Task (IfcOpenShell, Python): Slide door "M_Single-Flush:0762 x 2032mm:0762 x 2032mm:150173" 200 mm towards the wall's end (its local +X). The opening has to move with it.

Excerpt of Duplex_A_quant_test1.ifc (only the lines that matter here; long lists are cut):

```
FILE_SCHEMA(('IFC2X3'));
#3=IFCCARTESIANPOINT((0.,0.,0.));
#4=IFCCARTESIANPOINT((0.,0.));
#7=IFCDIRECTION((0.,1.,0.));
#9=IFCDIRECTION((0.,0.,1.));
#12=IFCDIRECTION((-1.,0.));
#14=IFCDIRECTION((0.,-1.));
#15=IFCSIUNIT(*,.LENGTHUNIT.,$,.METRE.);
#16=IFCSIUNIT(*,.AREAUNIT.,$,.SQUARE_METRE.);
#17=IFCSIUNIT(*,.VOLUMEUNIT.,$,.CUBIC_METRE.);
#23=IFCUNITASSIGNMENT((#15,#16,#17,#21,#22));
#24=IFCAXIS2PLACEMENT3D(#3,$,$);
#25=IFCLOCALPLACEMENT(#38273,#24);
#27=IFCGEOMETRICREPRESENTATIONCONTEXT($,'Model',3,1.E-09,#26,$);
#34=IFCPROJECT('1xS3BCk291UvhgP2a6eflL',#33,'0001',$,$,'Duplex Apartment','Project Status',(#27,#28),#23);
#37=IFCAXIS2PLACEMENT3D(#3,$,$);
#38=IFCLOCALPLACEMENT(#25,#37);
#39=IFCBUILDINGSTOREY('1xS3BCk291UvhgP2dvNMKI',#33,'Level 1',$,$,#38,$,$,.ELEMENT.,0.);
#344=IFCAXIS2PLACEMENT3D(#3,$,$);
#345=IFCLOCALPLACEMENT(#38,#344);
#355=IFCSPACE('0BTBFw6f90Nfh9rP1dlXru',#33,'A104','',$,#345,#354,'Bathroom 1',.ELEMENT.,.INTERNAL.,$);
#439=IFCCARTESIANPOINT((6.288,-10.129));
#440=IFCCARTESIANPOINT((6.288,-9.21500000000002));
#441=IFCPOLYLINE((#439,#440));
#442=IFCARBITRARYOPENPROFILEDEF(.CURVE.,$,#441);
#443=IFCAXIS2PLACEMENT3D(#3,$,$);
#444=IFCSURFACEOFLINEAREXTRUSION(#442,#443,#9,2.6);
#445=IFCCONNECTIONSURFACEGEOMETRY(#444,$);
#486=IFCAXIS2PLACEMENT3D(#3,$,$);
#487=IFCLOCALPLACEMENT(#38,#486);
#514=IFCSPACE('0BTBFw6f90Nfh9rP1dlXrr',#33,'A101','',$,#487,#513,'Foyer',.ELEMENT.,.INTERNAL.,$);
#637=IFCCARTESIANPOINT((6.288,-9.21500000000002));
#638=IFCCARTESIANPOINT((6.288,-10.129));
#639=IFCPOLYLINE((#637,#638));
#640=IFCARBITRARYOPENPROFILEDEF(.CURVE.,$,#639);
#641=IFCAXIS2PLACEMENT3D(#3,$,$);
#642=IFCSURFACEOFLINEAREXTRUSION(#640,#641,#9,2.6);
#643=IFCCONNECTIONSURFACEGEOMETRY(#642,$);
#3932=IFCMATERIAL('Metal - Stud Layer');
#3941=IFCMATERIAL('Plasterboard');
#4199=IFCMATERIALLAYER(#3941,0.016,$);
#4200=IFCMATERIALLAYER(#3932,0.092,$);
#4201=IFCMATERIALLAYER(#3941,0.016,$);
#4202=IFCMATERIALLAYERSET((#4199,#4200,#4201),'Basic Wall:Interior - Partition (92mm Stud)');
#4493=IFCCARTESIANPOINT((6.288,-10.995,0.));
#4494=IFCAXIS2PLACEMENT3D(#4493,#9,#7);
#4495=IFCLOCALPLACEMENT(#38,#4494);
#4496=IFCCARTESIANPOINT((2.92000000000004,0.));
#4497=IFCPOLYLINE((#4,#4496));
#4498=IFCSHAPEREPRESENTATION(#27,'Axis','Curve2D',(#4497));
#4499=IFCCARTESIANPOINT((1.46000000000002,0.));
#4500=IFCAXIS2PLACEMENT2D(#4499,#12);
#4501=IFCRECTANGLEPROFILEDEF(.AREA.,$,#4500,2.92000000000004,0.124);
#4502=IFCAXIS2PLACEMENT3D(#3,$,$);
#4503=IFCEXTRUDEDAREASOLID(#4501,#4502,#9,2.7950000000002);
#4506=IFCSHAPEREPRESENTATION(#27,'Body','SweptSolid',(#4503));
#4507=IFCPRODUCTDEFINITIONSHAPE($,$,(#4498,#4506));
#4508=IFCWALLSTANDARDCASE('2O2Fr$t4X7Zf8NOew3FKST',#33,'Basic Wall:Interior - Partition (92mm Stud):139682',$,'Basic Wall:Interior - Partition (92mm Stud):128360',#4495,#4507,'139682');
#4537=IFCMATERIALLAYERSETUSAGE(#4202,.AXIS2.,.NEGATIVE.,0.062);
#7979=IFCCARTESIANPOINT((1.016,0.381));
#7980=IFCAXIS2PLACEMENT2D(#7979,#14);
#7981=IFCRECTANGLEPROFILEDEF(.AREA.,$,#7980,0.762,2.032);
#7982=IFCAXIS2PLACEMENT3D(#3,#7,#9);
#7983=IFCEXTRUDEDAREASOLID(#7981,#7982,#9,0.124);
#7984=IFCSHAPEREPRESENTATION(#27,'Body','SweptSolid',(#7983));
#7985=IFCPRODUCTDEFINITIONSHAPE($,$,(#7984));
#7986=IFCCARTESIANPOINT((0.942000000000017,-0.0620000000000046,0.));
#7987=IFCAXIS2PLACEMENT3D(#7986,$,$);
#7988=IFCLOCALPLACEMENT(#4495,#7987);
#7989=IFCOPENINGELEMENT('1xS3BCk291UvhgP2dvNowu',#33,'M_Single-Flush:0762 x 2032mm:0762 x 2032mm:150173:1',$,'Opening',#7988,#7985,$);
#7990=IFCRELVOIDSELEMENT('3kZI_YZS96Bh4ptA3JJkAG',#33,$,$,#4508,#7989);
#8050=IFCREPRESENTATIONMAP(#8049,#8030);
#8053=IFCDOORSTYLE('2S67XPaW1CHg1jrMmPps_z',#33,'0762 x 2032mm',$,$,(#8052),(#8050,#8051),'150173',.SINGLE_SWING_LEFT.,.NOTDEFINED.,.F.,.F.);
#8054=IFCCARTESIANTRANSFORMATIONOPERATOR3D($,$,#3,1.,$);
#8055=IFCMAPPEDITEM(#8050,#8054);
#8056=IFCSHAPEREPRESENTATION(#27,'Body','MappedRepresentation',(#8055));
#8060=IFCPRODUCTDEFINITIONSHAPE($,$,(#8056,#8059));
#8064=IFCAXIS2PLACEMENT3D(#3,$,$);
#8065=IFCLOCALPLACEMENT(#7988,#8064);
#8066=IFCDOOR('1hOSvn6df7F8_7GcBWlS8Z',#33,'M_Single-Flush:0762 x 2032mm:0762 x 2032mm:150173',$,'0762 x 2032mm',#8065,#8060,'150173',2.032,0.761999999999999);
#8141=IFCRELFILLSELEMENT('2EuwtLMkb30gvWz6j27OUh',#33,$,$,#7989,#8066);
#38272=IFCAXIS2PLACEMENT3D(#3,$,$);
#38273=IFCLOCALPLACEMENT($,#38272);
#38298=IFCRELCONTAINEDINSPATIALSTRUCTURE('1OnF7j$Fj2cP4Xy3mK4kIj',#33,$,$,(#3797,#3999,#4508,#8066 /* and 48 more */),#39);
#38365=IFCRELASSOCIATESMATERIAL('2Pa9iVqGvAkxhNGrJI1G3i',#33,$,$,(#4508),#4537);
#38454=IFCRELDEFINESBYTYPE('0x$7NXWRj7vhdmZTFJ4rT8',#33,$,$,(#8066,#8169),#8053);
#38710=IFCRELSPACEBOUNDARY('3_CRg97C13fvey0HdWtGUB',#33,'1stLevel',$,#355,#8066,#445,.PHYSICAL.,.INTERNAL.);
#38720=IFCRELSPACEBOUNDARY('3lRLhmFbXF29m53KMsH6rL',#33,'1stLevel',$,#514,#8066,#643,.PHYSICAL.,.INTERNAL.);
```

```python
import numpy as np
import ifcopenshell
import ifcopenshell.api.geometry
import ifcopenshell.util.placement
import ifcopenshell.util.unit

model = ifcopenshell.open("Duplex_A_quant_test1.ifc")
unit_scale = ifcopenshell.util.unit.calculate_unit_scale(model)

door = model.by_guid("1hOSvn6df7F8_7GcBWlS8Z")
opening = door.FillsVoids[0].RelatingOpeningElement
wall = opening.VoidsElements[0].RelatingBuildingElement

wall_matrix = ifcopenshell.util.placement.get_local_placement(wall.ObjectPlacement)
shift = wall_matrix[:3, 0] * 0.2 / unit_scale
before = ifcopenshell.util.placement.get_local_placement(door.ObjectPlacement)[:3, 3].copy()

# The door is placed relative to its opening, so it follows when the opening moves.
matrix = ifcopenshell.util.placement.get_local_placement(opening.ObjectPlacement)
matrix[:3, 3] += shift
ifcopenshell.api.geometry.edit_object_placement(
    model, product=opening, matrix=matrix, is_si=False, should_transform_children=True
)

# Space boundary surfaces are stored in each space's coordinates; move them too.
for rel in door.ProvidesBoundaries:
    if not rel.ConnectionGeometry:
        continue
    surface = rel.ConnectionGeometry.SurfaceOnRelatingElement
    space_matrix = ifcopenshell.util.placement.get_local_placement(rel.RelatingSpace.ObjectPlacement)
    point = np.array(surface.Position.Location.Coordinates) + space_matrix[:3, :3].T @ shift
    surface.Position = model.createIfcAxis2Placement3D(
        model.createIfcCartesianPoint(point.tolist()), surface.Position.Axis, surface.Position.RefDirection
    )

after = ifcopenshell.util.placement.get_local_placement(door.ObjectPlacement)[:3, 3]
print("door moved by", (after - before).round(3) + 0.0)

model.write("Duplex_A_quant_test1_v2.ifc")
```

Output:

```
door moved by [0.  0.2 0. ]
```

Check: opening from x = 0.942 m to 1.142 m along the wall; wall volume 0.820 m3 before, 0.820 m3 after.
